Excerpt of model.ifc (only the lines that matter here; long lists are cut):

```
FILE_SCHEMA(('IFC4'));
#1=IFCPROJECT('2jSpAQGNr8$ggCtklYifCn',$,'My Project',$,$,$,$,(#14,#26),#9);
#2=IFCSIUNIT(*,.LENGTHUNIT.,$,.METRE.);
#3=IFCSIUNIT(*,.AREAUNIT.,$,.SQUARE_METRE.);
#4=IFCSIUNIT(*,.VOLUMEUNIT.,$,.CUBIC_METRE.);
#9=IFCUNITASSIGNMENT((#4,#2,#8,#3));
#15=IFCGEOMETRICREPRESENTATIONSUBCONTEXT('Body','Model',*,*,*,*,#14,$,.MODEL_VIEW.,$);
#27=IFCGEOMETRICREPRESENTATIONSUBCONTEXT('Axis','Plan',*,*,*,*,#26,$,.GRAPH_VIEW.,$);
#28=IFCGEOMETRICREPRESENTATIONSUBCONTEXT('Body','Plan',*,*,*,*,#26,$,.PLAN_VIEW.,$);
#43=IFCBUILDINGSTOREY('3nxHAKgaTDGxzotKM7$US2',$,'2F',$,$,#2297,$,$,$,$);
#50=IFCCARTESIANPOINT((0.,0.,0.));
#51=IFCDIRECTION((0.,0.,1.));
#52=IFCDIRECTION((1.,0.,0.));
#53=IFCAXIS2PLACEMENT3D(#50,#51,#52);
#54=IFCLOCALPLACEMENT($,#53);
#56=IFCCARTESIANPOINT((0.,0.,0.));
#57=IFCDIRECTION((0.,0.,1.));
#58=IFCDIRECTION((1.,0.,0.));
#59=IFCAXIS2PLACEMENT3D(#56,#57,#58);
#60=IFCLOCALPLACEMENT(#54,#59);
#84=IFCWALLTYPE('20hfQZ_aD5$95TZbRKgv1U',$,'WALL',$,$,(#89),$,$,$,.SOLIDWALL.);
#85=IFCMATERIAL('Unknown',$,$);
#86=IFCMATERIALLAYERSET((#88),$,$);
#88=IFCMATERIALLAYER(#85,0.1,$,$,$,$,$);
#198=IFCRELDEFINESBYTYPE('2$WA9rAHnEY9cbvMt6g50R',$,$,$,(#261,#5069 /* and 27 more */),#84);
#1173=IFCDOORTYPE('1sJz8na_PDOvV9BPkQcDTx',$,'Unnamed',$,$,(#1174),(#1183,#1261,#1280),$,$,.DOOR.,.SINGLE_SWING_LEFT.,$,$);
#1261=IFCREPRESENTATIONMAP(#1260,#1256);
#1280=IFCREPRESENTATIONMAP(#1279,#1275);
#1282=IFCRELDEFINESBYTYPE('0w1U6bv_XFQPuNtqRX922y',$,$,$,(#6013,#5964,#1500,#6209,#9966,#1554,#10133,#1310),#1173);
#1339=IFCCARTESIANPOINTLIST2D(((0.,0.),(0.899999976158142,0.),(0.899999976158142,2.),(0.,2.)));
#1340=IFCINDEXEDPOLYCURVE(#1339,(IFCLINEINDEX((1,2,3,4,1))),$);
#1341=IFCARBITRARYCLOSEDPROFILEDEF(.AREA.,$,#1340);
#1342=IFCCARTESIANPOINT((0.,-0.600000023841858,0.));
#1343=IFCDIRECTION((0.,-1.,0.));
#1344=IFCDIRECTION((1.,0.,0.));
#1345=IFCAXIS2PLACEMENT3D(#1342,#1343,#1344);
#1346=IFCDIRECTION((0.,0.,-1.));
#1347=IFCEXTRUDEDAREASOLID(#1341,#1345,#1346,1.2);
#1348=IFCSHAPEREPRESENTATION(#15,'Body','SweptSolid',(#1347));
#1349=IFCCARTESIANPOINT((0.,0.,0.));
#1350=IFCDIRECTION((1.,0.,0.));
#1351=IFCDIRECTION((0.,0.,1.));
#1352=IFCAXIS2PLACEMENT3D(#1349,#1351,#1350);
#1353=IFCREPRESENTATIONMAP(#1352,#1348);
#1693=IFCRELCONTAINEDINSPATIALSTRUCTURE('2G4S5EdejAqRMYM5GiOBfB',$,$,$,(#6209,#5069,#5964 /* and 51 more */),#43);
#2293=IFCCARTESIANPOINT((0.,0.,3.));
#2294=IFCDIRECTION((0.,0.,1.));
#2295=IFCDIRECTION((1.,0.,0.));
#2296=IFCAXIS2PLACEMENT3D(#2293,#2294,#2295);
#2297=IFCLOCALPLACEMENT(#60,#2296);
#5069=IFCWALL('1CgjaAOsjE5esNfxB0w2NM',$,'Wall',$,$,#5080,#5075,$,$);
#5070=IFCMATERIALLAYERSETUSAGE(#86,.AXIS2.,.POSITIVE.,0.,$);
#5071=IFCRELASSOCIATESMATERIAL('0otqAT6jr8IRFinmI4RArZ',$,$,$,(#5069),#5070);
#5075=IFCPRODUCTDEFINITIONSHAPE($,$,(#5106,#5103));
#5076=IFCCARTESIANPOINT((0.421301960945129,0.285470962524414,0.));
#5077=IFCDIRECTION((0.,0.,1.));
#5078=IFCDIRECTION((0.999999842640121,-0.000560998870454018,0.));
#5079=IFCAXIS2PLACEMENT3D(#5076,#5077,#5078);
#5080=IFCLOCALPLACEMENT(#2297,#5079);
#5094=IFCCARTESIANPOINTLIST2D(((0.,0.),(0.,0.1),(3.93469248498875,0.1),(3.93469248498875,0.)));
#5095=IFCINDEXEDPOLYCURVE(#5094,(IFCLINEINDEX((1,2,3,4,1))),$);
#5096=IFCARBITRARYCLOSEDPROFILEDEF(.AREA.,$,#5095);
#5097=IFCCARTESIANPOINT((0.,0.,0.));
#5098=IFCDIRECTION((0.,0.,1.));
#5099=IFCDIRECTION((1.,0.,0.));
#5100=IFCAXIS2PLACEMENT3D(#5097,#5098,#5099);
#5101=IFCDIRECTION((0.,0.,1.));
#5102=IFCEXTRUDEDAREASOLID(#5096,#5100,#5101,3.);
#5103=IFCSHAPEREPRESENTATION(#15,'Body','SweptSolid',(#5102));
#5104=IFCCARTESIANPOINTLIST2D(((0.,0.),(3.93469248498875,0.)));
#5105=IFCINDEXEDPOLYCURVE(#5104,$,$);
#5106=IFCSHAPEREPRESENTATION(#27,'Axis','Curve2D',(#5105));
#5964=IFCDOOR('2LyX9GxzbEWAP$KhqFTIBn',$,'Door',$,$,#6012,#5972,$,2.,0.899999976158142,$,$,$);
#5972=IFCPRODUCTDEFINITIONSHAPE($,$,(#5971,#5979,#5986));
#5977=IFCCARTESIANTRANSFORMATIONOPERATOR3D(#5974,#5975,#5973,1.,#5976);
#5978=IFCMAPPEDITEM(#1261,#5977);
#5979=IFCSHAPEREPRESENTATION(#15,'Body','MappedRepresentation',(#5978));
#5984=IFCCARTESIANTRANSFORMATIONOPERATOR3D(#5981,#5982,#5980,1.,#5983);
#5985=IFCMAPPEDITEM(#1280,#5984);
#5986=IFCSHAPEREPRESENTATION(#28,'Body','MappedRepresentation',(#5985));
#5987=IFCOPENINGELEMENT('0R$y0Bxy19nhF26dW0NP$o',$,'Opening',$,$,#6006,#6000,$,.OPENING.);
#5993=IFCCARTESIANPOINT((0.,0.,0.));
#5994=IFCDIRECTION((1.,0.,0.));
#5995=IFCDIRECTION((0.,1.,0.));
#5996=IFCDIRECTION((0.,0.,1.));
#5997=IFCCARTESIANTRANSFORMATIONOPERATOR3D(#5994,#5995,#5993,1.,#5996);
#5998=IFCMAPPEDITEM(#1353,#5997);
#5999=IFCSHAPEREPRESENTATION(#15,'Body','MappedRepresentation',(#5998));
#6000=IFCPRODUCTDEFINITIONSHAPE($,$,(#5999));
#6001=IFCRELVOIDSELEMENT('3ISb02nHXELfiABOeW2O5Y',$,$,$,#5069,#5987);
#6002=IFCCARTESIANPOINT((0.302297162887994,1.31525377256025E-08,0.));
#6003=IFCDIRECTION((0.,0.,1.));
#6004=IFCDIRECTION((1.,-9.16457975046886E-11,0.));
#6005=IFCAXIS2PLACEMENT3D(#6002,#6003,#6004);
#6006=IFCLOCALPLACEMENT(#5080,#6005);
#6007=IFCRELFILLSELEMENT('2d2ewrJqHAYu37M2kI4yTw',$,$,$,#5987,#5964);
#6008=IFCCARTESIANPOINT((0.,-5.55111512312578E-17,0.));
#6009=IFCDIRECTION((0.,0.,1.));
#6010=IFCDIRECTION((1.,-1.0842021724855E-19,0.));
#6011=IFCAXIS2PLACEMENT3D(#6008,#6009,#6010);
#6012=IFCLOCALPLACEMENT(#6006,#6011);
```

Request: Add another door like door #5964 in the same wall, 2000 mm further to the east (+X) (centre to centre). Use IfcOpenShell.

```python
import ifcopenshell
import ifcopenshell.api.feature
import ifcopenshell.api.geometry
import ifcopenshell.api.root
import ifcopenshell.geom
import ifcopenshell.util.element
import ifcopenshell.util.placement
import ifcopenshell.util.shape
import ifcopenshell.util.unit

model = ifcopenshell.open("model.ifc")
unit_scale = ifcopenshell.util.unit.calculate_unit_scale(model)
settings = ifcopenshell.geom.settings()


def volume(element):
    """Net volume in cubic metres, openings subtracted."""
    shape = ifcopenshell.geom.create_shape(settings, element)
    return ifcopenshell.util.shape.get_volume(shape.geometry)


door = model.by_guid("2LyX9GxzbEWAP$KhqFTIBn")
opening = door.FillsVoids[0].RelatingOpeningElement
wall = opening.VoidsElements[0].RelatingBuildingElement
before = volume(wall)
shift = ifcopenshell.util.placement.get_local_placement(wall.ObjectPlacement)[:3, 0] * 2 / unit_scale

# copy_class copies the void relationship, type, container and properties, but no geometry.
new_opening = ifcopenshell.api.root.copy_class(model, product=opening)
new_opening.Representation = ifcopenshell.util.element.copy_deep(
    model, opening.Representation, exclude=["IfcGeometricRepresentationContext", "IfcRepresentationMap"]
)
new_door = ifcopenshell.api.root.copy_class(model, product=door)
new_door.Representation = ifcopenshell.util.element.copy_deep(
    model, door.Representation, exclude=["IfcGeometricRepresentationContext", "IfcRepresentationMap"]
)
ifcopenshell.api.feature.add_filling(model, opening=new_opening, element=new_door)

for old, new in ((opening, new_opening), (door, new_door)):
    matrix = ifcopenshell.util.placement.get_local_placement(old.ObjectPlacement)
    matrix[:3, 3] += shift
    ifcopenshell.api.geometry.edit_object_placement(model, product=new, matrix=matrix, is_si=False)

after = volume(wall)

print(f"wall volume {before:.3f} -> {after:.3f} m3")

model.write("model_edited.ifc")
```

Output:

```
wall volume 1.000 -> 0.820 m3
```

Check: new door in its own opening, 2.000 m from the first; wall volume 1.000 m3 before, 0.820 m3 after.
